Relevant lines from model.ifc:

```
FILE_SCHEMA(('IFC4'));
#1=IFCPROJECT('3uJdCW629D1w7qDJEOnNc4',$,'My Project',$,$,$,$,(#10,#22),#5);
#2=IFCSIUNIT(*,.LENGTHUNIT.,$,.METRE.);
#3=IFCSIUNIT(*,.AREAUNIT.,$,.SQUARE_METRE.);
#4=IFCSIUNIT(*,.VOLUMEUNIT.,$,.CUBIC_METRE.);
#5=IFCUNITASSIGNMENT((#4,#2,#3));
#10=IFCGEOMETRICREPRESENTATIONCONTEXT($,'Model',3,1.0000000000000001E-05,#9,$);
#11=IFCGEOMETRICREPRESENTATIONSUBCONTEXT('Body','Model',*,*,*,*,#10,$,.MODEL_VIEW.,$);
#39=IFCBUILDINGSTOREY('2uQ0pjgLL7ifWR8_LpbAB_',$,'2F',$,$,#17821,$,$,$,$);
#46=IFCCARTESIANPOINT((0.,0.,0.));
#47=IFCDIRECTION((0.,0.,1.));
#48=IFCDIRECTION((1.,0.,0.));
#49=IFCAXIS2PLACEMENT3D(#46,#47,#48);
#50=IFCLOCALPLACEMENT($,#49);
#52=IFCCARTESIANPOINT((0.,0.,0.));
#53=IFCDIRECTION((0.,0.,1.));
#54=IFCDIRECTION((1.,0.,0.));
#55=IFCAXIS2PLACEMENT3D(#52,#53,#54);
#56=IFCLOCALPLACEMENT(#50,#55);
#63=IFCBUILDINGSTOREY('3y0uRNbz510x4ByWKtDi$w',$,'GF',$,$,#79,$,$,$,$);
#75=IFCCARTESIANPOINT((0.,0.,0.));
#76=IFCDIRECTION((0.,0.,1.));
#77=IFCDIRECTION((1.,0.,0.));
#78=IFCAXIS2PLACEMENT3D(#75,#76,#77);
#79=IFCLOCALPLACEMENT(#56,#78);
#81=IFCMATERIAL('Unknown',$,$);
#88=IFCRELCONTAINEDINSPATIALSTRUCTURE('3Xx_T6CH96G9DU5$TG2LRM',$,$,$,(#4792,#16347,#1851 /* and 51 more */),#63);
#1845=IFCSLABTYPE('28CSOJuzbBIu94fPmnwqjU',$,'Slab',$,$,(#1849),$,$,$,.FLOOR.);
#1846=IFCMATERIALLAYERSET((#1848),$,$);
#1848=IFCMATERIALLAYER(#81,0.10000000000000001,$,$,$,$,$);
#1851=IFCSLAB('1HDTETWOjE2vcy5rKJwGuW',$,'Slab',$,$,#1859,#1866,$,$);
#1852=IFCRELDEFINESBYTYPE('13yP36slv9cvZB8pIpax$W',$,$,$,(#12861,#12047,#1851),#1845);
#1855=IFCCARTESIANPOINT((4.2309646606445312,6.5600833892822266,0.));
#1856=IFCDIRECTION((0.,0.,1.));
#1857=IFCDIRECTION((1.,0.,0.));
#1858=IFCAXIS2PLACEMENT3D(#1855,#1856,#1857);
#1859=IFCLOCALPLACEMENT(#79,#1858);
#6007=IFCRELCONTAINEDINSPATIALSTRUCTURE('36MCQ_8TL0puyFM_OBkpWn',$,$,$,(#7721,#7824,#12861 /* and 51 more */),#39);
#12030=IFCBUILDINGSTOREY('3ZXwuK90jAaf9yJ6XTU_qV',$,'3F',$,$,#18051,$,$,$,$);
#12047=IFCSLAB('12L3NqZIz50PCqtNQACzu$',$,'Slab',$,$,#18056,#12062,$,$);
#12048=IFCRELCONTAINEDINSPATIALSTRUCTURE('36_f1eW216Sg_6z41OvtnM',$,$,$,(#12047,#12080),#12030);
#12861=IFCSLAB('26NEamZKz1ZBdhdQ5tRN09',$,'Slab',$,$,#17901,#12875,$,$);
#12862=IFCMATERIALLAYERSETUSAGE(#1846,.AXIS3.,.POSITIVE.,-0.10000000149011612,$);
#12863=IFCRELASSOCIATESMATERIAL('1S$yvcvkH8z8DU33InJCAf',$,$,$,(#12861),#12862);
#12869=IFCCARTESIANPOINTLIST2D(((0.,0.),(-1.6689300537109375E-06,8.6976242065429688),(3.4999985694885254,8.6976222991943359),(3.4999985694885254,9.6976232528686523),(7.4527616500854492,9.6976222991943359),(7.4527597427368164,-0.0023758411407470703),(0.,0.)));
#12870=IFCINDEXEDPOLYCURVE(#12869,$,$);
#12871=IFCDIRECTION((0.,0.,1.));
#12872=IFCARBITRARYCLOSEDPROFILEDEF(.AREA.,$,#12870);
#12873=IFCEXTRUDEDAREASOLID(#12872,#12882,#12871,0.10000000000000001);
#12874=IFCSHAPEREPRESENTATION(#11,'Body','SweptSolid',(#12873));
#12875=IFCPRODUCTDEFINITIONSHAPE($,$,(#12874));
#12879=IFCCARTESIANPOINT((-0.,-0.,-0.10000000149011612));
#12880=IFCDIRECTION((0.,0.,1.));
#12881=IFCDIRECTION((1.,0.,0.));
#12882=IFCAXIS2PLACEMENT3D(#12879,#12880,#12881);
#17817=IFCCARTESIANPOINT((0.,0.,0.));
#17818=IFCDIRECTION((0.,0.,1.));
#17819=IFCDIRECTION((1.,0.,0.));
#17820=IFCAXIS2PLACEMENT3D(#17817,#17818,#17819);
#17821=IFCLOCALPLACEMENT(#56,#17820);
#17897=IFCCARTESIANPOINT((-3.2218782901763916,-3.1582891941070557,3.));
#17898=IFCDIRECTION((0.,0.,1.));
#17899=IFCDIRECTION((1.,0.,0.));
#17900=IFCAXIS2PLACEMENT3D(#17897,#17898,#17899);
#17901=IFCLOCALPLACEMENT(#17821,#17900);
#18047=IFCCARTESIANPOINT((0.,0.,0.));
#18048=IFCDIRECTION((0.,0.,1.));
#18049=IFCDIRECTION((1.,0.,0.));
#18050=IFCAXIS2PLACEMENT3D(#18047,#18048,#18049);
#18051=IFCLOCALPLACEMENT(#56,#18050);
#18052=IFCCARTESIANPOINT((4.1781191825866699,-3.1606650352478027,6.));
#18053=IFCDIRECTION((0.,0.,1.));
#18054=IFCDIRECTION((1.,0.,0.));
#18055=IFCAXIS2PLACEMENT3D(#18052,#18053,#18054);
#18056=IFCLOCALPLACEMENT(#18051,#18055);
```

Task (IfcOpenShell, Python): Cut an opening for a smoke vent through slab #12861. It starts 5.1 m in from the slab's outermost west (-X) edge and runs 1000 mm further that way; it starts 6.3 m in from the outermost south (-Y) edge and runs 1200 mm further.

```python
import numpy as np
import ifcopenshell
import ifcopenshell.api.feature
import ifcopenshell.api.geometry
import ifcopenshell.api.root
import ifcopenshell.geom
import ifcopenshell.util.placement
import ifcopenshell.util.representation
import ifcopenshell.util.shape
import ifcopenshell.util.unit

model = ifcopenshell.open("model.ifc")
unit_scale = ifcopenshell.util.unit.calculate_unit_scale(model)
settings = ifcopenshell.geom.settings()


def volume(element):
    """Net volume in cubic metres, openings subtracted."""
    shape = ifcopenshell.geom.create_shape(settings, element)
    return ifcopenshell.util.shape.get_volume(shape.geometry)


slab = model.by_guid("26NEamZKz1ZBdhdQ5tRN09")
before = volume(slab)

# Extent in the slab's own axes, in metres. The edges named are its -X and -Y sides.
slab_shape = ifcopenshell.geom.create_shape(settings, slab)
vertices = ifcopenshell.util.shape.get_vertices(slab_shape.geometry)
x_min, y_min, bottom = vertices.min(axis=0)
top = vertices[:, 2].max()

opening = ifcopenshell.api.root.create_entity(model, ifc_class="IfcOpeningElement", name="Smoke vent opening", predefined_type="OPENING")
context = ifcopenshell.util.representation.get_context(model, "Model", "Body", "MODEL_VIEW")
width, depth = 1, 1.2
outline = [(0.0, 0.0), (width, 0.0), (width, depth), (0.0, depth), (0.0, 0.0)]
# Overshoot both faces by 50 mm so the cut is clean.
shape = ifcopenshell.api.geometry.add_slab_representation(
    model, context=context, depth=top - bottom + 0.1, polyline=outline
)
ifcopenshell.api.geometry.assign_representation(model, product=opening, representation=shape)

matrix = ifcopenshell.util.placement.get_local_placement(slab.ObjectPlacement)
matrix[:, 3] = matrix @ np.append(np.array([x_min + 5.1, y_min + 6.3, bottom - 0.05]) / unit_scale, 1.0)
ifcopenshell.api.geometry.edit_object_placement(model, product=opening, matrix=matrix, is_si=False)
ifcopenshell.api.feature.add_feature(model, feature=opening, element=slab)

after = volume(slab)

print(f"slab volume {before:.3f} -> {after:.3f} m3")

model.write("model_rev.ifc")
```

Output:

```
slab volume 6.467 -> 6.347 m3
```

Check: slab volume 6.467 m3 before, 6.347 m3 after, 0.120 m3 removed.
